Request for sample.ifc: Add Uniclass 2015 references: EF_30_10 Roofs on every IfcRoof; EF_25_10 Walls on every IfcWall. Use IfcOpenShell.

First a look at what the model holds.

```python
import ifcopenshell

model = ifcopenshell.open("sample.ifc")
print(model.schema)
print("classifications:", [c.Name for c in model.by_type("IfcClassification")])
for ifc_class in ("IfcDoor", "IfcRoof", "IfcStair", "IfcWall", "IfcWindow"):
    print(ifc_class, len(model.by_type(ifc_class)))
```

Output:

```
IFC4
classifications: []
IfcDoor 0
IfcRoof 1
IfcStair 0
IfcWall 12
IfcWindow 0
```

```python
import ifcopenshell
import ifcopenshell.api.classification

model = ifcopenshell.open("sample.ifc")

system = ifcopenshell.api.classification.add_classification(model, classification="Uniclass 2015")

codes = {
    "IfcRoof": ("EF_30_10", "Roofs"),
    "IfcWall": ("EF_25_10", "Walls"),
}
for ifc_class, (code, name) in codes.items():
    products = model.by_type(ifc_class)
    ifcopenshell.api.classification.add_reference(
        model, products=products, classification=system, identification=code, name=name
    )
    print(code, len(products))

model.write("sample_rev.ifc")
```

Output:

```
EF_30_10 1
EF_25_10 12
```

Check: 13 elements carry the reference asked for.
